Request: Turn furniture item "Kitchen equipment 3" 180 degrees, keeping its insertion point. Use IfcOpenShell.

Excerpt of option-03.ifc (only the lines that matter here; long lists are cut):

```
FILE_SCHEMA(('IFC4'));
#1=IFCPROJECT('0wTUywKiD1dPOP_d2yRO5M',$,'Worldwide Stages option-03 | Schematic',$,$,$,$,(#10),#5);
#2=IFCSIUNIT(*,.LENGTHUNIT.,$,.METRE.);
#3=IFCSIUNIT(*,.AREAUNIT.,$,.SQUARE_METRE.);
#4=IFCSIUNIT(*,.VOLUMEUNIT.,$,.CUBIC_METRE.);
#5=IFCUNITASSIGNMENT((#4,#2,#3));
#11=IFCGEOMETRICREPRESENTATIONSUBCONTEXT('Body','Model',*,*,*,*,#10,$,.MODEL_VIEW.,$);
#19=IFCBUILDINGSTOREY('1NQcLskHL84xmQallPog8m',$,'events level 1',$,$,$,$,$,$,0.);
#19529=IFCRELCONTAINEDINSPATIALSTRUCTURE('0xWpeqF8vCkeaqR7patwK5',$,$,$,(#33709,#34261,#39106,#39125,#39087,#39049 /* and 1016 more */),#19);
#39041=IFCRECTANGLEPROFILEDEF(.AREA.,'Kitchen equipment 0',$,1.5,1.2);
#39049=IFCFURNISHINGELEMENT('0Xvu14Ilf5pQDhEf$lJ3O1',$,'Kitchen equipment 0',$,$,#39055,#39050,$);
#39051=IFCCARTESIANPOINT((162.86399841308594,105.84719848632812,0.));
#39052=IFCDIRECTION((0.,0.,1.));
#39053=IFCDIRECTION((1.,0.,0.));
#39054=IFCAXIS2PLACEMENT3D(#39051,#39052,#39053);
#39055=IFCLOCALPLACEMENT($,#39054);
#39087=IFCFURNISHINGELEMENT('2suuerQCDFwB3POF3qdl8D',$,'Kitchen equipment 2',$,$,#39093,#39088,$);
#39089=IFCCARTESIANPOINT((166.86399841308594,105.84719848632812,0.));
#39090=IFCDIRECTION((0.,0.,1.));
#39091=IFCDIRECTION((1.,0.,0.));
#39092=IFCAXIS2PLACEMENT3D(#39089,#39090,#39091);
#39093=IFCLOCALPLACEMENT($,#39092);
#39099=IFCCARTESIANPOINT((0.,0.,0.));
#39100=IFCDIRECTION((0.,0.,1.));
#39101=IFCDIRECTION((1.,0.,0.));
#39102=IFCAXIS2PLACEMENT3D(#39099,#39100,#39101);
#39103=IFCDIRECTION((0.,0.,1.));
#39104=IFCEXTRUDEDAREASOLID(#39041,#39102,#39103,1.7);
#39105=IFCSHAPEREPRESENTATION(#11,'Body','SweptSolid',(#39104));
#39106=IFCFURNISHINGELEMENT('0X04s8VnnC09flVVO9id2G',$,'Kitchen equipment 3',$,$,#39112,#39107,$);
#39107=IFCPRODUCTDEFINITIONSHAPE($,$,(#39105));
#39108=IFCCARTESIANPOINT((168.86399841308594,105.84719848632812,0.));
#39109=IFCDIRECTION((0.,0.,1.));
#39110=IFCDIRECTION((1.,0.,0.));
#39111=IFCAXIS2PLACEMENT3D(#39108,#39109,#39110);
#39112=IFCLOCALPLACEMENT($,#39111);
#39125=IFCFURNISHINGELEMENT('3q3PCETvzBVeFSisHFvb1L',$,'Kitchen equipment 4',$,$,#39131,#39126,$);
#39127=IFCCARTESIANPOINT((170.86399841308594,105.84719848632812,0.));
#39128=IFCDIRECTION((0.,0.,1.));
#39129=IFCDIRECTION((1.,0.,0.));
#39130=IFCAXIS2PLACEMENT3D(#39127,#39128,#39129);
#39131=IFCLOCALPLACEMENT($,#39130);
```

```python
import ifcopenshell
import ifcopenshell.api.geometry
import ifcopenshell.util.placement

model = ifcopenshell.open("option-03.ifc")

item = model.by_guid("0X04s8VnnC09flVVO9id2G")
matrix = ifcopenshell.util.placement.get_local_placement(item.ObjectPlacement)
matrix = matrix @ ifcopenshell.util.placement.rotation(180, "Z")
ifcopenshell.api.geometry.edit_object_placement(model, product=item, matrix=matrix, is_si=False)

print(ifcopenshell.util.placement.get_local_placement(item.ObjectPlacement).round(3) + 0.0)

model.write("option-03_updated.ifc")
```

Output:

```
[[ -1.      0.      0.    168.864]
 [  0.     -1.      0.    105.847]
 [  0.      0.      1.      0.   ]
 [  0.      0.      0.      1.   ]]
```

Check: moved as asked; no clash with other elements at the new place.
